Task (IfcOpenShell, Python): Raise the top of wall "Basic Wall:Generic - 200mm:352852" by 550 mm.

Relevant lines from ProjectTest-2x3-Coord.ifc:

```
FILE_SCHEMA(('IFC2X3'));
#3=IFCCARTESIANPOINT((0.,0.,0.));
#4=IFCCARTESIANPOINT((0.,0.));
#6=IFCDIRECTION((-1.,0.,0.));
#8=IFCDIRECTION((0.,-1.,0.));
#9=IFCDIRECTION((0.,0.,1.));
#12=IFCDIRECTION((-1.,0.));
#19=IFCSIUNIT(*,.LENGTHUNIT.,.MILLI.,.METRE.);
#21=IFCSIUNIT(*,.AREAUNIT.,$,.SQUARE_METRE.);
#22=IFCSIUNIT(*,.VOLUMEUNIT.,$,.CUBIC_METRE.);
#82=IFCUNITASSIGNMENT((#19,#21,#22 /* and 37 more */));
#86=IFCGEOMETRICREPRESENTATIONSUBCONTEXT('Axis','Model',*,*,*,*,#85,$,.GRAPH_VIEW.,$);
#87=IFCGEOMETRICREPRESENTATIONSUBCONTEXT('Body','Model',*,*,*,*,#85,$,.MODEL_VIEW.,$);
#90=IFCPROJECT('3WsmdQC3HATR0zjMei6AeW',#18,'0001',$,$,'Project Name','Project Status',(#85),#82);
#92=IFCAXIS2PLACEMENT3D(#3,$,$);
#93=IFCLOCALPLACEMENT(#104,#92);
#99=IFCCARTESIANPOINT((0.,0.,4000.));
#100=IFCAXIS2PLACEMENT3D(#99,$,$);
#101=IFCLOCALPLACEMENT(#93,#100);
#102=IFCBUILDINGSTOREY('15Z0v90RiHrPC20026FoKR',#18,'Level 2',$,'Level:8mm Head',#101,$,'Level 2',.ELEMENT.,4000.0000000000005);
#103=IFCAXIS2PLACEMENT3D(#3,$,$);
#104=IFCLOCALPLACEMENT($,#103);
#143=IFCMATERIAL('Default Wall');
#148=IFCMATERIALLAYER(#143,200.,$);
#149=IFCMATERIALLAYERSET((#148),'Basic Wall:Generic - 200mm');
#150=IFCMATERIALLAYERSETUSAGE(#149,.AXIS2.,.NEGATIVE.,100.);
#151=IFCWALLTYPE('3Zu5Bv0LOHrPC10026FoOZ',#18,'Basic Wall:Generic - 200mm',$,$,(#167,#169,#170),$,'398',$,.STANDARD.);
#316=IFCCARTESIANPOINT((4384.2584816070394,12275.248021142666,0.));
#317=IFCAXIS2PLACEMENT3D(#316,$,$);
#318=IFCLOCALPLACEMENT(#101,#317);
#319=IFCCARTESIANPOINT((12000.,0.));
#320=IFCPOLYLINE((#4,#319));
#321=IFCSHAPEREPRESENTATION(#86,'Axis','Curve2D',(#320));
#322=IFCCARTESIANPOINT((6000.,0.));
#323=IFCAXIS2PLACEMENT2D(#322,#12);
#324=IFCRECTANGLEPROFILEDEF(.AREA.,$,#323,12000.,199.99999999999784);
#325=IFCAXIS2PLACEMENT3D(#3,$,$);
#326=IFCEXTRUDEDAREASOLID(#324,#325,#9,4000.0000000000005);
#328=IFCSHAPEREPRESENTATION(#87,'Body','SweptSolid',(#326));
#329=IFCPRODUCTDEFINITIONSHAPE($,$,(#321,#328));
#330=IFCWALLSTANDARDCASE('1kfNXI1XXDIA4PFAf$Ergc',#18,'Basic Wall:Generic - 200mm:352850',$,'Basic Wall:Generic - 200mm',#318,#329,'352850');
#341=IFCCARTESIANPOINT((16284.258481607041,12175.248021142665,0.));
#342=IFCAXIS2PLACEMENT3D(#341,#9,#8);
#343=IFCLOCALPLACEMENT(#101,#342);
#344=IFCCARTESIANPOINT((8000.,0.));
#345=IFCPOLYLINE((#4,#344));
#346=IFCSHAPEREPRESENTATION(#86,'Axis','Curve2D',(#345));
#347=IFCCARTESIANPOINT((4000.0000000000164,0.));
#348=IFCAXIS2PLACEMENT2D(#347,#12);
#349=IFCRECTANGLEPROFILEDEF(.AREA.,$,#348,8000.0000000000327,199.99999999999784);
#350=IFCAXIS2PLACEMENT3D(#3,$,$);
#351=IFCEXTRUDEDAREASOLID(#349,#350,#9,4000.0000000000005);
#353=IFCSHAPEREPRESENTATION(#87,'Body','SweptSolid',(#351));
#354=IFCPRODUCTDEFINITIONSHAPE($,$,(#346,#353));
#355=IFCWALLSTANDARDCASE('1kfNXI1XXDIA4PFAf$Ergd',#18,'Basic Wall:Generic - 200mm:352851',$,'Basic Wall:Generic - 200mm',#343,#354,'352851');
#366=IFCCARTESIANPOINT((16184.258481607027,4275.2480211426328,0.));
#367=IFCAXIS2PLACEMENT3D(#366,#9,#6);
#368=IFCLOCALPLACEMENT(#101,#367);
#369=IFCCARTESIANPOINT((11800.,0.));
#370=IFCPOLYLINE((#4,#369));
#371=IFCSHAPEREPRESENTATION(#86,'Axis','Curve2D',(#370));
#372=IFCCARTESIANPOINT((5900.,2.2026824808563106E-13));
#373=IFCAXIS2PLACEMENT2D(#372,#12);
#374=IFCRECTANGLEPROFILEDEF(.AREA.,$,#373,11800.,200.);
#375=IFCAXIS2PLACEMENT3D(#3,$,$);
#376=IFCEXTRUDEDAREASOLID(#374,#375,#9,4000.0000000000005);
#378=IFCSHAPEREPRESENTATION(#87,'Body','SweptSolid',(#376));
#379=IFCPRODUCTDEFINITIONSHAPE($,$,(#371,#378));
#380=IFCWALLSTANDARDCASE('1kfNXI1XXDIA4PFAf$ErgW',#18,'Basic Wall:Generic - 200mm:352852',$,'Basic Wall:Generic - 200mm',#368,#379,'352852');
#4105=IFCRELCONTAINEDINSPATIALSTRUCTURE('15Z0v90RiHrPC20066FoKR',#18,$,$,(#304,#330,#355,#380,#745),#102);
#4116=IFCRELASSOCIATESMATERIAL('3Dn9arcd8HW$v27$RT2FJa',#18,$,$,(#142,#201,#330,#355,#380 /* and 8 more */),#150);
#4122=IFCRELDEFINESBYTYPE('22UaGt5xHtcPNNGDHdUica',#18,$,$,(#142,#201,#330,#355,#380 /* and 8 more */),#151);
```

```python
import ifcopenshell
import ifcopenshell.geom
import ifcopenshell.util.representation
import ifcopenshell.util.shape
import ifcopenshell.util.unit

model = ifcopenshell.open("ProjectTest-2x3-Coord.ifc")
unit_scale = ifcopenshell.util.unit.calculate_unit_scale(model)
settings = ifcopenshell.geom.settings()


def volume(element):
    """Net volume in cubic metres, openings subtracted."""
    shape = ifcopenshell.geom.create_shape(settings, element)
    return ifcopenshell.util.shape.get_volume(shape.geometry)


wall = model.by_guid("1kfNXI1XXDIA4PFAf$ErgW")
before = volume(wall)

body = ifcopenshell.util.representation.get_representation(wall, "Model", "Body")
solid = body.Items[0]
old_height = solid.Depth
solid.Depth += 0.55 / unit_scale
after = volume(wall)

print(f"height {old_height:g} -> {solid.Depth:g}, volume {before:.3f} -> {after:.3f} m3")

model.write("ProjectTest-2x3-Coord_edited.ifc")
```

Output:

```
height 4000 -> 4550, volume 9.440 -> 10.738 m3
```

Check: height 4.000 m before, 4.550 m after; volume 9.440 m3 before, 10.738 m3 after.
